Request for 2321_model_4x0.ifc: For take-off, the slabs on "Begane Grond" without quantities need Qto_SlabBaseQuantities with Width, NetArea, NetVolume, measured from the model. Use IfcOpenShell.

First a look at what the model holds.

```python
import ifcopenshell
import ifcopenshell.util.element
import ifcopenshell.util.unit

model = ifcopenshell.open("2321_model_4x0.ifc")
print(model.schema)
for unit_type in ("LENGTHUNIT", "AREAUNIT", "VOLUMEUNIT"):
    print(unit_type, ifcopenshell.util.unit.calculate_unit_scale(model, unit_type))
storey = next(s for s in model.by_type("IfcBuildingStorey") if s.Name == "Begane Grond")
slabs = [e for e in ifcopenshell.util.element.get_decomposition(storey) if e.is_a("IfcSlab")]
for e in sorted(slabs, key=lambda e: e.id()):
    print(e.id(), e.is_a(), e.Name, list(ifcopenshell.util.element.get_psets(e, qtos_only=True)), sep=" | ")
```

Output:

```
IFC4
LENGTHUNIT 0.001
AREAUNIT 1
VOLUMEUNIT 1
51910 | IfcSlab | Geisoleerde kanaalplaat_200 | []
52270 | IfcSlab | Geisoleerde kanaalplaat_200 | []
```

```python
import ifcopenshell
import ifcopenshell.api.pset
import ifcopenshell.geom
import ifcopenshell.util.element
import ifcopenshell.util.shape
import ifcopenshell.util.unit

model = ifcopenshell.open("2321_model_4x0.ifc")
unit_scale = ifcopenshell.util.unit.calculate_unit_scale(model)
area_scale = ifcopenshell.util.unit.calculate_unit_scale(model, "AREAUNIT")
volume_scale = ifcopenshell.util.unit.calculate_unit_scale(model, "VOLUMEUNIT")
settings = ifcopenshell.geom.settings()

storey = next(s for s in model.by_type("IfcBuildingStorey") if s.Name == "Begane Grond")
slabs = [e for e in ifcopenshell.util.element.get_decomposition(storey) if e.is_a("IfcSlab")]

for e in sorted(slabs, key=lambda e: e.id()):
    if ifcopenshell.util.element.get_psets(e, qtos_only=True, should_inherit=False):
        continue
    # Geometry comes back in metres, in the element's own axes.
    shape = ifcopenshell.geom.create_shape(settings, e)
    values = {
        "Width": ifcopenshell.util.shape.get_z(shape.geometry) / unit_scale,
        "NetArea": ifcopenshell.util.shape.get_footprint_area(shape.geometry) / area_scale,
        "NetVolume": ifcopenshell.util.shape.get_volume(shape.geometry) / volume_scale,
    }
    qto = ifcopenshell.api.pset.add_qto(model, product=e, name="Qto_SlabBaseQuantities")
    ifcopenshell.api.pset.edit_qto(model, qto=qto, properties=values)
    print(e.id(), {k: round(v, 3) for k, v in values.items()})

model.write("2321_model_4x0_rev.ifc")
```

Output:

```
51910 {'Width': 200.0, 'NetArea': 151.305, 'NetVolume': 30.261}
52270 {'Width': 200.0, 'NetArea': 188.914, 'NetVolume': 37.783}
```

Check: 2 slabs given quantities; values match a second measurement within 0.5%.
